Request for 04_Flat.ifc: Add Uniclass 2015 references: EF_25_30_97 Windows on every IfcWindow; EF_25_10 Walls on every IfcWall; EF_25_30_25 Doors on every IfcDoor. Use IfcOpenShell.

First a look at what the model holds.

```python
import ifcopenshell

model = ifcopenshell.open("04_Flat.ifc")
print(model.schema)
print("classifications:", [c.Name for c in model.by_type("IfcClassification")])
for ifc_class in ("IfcDoor", "IfcRoof", "IfcStair", "IfcWall", "IfcWindow"):
    print(ifc_class, len(model.by_type(ifc_class)))
```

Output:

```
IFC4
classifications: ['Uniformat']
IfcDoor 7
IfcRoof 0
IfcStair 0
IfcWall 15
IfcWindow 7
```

```python
import ifcopenshell
import ifcopenshell.api.classification

model = ifcopenshell.open("04_Flat.ifc")

system = ifcopenshell.api.classification.add_classification(model, classification="Uniclass 2015")

codes = {
    "IfcWindow": ("EF_25_30_97", "Windows"),
    "IfcWall": ("EF_25_10", "Walls"),
    "IfcDoor": ("EF_25_30_25", "Doors"),
}
for ifc_class, (code, name) in codes.items():
    products = model.by_type(ifc_class)
    ifcopenshell.api.classification.add_reference(
        model, products=products, classification=system, identification=code, name=name
    )
    print(code, len(products))

model.write("04_Flat_v2.ifc")
```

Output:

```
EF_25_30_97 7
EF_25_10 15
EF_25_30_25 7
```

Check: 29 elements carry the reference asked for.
